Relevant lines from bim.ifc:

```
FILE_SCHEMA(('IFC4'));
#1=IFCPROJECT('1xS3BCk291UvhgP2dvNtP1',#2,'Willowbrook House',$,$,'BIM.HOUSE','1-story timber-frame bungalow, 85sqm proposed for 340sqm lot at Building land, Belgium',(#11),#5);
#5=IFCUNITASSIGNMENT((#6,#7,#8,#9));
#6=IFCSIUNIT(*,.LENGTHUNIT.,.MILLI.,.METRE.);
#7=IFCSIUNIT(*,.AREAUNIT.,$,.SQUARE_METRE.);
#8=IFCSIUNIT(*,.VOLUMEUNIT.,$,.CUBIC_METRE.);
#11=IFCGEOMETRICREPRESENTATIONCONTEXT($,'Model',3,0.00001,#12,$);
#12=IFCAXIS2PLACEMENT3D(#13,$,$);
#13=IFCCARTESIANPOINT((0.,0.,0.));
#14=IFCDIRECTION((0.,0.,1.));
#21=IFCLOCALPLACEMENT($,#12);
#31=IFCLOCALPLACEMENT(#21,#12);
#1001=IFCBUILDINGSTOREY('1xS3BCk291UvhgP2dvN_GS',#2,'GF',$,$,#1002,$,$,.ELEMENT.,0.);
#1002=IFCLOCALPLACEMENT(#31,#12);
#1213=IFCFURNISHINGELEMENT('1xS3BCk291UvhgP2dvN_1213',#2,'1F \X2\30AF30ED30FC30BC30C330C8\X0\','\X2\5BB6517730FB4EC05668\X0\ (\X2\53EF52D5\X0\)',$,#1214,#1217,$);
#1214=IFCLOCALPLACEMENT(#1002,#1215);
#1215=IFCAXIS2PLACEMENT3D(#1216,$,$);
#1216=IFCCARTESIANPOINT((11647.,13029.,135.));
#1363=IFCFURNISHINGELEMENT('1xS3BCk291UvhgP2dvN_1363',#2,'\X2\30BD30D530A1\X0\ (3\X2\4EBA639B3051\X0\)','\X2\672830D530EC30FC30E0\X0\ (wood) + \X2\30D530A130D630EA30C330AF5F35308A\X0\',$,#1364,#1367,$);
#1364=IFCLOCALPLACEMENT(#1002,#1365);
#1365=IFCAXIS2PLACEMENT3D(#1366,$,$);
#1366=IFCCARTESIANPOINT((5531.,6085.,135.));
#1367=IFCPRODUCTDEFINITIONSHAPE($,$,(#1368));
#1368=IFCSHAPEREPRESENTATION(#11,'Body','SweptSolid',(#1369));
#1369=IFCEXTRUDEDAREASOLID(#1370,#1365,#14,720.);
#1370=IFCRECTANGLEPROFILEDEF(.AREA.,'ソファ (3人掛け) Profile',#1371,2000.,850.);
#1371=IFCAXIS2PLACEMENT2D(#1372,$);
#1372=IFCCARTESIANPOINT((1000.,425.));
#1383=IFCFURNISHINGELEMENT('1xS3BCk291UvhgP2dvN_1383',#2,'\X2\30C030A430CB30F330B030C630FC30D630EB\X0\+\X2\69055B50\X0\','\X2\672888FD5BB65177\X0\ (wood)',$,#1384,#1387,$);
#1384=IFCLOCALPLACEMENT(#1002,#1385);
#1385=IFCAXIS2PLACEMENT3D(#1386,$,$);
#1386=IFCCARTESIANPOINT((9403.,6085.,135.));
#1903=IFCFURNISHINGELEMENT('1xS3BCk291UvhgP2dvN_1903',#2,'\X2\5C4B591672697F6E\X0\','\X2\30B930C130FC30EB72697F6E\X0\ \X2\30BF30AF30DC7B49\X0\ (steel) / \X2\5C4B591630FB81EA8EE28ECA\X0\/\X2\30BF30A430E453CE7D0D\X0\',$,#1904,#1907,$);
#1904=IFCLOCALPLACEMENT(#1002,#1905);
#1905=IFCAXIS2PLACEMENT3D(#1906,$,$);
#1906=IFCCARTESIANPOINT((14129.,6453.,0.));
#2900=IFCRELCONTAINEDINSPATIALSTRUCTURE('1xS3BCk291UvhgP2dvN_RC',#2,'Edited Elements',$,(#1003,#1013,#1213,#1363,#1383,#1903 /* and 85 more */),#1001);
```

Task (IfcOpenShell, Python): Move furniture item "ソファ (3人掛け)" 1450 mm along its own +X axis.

```python
import ifcopenshell
import ifcopenshell.api.geometry
import ifcopenshell.util.placement

model = ifcopenshell.open("bim.ifc")

item = model.by_id(1363)
matrix = ifcopenshell.util.placement.get_local_placement(item.ObjectPlacement)
matrix[:3, 3] += matrix[:3, 0] * 1450.0
ifcopenshell.api.geometry.edit_object_placement(model, product=item, matrix=matrix, is_si=False)

print(ifcopenshell.util.placement.get_local_placement(item.ObjectPlacement).round(3) + 0.0)

model.write("bim_edited.ifc")
```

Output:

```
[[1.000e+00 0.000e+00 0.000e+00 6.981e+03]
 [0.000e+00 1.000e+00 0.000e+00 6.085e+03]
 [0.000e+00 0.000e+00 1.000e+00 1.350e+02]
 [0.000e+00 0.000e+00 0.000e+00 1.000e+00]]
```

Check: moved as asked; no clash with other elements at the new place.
